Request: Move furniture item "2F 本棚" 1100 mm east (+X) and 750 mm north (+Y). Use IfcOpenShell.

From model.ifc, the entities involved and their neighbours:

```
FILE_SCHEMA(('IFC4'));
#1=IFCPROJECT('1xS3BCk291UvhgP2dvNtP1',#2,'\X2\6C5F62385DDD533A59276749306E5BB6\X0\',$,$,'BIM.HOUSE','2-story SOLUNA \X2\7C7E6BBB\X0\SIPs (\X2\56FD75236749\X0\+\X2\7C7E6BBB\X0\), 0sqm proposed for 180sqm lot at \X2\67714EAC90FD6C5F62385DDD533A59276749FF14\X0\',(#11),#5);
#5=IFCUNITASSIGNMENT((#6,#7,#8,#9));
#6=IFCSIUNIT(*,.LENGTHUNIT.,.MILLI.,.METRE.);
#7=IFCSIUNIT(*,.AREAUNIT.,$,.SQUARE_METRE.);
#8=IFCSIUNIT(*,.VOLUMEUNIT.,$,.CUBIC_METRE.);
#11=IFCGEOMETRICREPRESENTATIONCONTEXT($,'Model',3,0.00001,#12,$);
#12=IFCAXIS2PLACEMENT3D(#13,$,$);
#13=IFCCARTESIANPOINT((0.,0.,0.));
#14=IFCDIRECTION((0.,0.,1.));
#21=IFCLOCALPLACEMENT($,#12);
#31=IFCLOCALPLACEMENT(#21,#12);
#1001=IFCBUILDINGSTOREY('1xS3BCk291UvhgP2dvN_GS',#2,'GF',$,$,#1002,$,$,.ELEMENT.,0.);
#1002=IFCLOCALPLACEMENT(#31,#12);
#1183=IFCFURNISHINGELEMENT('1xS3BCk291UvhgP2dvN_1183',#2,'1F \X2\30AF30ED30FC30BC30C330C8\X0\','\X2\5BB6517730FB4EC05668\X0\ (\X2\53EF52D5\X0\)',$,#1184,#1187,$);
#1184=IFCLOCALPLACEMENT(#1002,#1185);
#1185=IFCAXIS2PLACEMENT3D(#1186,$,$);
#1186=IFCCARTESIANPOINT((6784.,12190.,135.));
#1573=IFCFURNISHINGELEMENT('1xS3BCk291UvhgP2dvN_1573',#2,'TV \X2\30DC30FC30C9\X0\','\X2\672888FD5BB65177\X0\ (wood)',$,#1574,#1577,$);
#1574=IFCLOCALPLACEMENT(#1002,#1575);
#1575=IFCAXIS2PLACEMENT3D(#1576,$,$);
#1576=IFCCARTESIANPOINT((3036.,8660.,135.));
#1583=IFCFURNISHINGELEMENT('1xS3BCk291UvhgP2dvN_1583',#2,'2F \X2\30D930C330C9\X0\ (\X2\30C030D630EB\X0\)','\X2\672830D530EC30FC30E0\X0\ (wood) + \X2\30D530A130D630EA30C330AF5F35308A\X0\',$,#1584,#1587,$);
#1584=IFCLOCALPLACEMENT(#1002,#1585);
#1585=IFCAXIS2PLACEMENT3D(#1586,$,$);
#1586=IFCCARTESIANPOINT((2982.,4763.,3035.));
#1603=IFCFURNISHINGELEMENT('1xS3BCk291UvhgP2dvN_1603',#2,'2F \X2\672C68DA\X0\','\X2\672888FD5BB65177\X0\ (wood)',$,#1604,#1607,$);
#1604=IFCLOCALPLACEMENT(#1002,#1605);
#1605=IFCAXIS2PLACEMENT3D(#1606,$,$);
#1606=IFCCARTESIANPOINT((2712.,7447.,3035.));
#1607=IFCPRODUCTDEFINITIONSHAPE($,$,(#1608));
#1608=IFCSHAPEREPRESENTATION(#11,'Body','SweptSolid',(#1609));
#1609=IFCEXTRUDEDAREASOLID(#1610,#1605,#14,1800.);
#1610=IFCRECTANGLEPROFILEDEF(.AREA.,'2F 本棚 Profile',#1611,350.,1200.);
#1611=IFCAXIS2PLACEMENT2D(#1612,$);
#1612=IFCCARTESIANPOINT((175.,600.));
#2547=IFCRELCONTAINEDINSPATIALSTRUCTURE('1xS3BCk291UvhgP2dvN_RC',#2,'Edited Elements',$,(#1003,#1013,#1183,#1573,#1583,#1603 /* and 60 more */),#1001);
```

```python
import ifcopenshell
import ifcopenshell.api.geometry
import ifcopenshell.util.placement

model = ifcopenshell.open("model.ifc")

item = model.by_guid("1xS3BCk291UvhgP2dvN_1603")
matrix = ifcopenshell.util.placement.get_local_placement(item.ObjectPlacement)
matrix[0, 3] += 1100.0
matrix[1, 3] += 750.0
ifcopenshell.api.geometry.edit_object_placement(model, product=item, matrix=matrix, is_si=False)

print(ifcopenshell.util.placement.get_local_placement(item.ObjectPlacement).round(3) + 0.0)

model.write("model_v2.ifc")
```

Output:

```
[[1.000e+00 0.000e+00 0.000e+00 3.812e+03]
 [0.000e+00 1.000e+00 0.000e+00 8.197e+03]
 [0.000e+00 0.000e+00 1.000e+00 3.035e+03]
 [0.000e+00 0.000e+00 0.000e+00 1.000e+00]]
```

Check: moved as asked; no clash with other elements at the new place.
